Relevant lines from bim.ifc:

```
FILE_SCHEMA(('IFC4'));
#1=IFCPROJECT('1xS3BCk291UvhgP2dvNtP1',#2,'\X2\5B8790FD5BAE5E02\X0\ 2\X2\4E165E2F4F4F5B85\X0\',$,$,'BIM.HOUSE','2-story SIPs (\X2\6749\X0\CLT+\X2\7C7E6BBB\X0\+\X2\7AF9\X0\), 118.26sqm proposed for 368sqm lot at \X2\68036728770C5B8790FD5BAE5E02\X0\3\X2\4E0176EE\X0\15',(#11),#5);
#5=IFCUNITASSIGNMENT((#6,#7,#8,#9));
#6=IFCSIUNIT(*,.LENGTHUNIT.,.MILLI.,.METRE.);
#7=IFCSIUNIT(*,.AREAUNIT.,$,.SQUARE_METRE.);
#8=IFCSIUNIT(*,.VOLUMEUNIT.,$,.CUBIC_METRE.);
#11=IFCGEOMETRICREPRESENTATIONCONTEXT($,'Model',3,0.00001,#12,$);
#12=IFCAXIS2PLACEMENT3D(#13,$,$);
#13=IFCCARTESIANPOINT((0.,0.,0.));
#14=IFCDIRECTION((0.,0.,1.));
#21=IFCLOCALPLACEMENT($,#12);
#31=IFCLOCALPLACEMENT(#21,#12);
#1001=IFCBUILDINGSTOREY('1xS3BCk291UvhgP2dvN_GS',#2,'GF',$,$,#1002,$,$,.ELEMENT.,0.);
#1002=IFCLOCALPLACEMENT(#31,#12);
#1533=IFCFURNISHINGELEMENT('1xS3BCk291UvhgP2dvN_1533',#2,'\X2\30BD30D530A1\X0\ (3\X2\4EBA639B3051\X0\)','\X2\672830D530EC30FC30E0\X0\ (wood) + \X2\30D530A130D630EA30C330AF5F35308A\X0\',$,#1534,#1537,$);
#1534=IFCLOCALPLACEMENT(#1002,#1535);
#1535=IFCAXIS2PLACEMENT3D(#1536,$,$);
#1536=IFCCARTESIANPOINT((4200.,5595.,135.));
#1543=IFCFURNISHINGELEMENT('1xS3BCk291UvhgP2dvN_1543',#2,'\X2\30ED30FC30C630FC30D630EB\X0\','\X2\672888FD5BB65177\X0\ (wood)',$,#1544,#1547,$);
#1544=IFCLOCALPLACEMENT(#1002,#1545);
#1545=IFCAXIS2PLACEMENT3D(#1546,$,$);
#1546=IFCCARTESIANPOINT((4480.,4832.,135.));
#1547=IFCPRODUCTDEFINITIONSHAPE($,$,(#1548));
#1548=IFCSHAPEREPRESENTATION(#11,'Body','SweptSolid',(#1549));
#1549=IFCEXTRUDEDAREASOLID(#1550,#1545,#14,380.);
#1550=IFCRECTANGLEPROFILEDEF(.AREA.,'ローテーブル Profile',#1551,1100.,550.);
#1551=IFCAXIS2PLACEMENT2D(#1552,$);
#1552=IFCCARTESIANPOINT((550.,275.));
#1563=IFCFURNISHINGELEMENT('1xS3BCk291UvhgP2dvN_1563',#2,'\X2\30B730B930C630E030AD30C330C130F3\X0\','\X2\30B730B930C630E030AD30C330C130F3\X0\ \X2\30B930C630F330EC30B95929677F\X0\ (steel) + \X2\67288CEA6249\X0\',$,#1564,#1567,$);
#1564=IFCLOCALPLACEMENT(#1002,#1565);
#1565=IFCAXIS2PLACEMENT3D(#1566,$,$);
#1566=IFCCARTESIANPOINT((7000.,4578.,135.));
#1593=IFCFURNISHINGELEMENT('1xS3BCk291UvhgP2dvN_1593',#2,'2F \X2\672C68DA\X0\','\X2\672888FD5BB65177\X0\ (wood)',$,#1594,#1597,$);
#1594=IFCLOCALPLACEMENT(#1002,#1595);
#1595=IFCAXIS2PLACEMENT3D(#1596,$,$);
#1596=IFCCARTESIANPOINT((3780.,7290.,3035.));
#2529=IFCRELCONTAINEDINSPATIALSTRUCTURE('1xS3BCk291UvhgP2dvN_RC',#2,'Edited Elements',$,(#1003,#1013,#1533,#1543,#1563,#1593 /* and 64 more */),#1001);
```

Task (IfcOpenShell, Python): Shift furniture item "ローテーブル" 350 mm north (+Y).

```python
import ifcopenshell
import ifcopenshell.api.geometry
import ifcopenshell.util.placement

model = ifcopenshell.open("bim.ifc")

item = model.by_guid("1xS3BCk291UvhgP2dvN_1543")
matrix = ifcopenshell.util.placement.get_local_placement(item.ObjectPlacement)
matrix[1, 3] += 350.0
ifcopenshell.api.geometry.edit_object_placement(model, product=item, matrix=matrix, is_si=False)

print(ifcopenshell.util.placement.get_local_placement(item.ObjectPlacement).round(3) + 0.0)

model.write("bim-out.ifc")
```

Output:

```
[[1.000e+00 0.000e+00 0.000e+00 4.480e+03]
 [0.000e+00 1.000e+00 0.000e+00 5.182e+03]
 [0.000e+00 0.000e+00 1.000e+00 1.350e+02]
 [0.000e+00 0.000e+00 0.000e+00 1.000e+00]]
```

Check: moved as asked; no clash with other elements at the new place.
